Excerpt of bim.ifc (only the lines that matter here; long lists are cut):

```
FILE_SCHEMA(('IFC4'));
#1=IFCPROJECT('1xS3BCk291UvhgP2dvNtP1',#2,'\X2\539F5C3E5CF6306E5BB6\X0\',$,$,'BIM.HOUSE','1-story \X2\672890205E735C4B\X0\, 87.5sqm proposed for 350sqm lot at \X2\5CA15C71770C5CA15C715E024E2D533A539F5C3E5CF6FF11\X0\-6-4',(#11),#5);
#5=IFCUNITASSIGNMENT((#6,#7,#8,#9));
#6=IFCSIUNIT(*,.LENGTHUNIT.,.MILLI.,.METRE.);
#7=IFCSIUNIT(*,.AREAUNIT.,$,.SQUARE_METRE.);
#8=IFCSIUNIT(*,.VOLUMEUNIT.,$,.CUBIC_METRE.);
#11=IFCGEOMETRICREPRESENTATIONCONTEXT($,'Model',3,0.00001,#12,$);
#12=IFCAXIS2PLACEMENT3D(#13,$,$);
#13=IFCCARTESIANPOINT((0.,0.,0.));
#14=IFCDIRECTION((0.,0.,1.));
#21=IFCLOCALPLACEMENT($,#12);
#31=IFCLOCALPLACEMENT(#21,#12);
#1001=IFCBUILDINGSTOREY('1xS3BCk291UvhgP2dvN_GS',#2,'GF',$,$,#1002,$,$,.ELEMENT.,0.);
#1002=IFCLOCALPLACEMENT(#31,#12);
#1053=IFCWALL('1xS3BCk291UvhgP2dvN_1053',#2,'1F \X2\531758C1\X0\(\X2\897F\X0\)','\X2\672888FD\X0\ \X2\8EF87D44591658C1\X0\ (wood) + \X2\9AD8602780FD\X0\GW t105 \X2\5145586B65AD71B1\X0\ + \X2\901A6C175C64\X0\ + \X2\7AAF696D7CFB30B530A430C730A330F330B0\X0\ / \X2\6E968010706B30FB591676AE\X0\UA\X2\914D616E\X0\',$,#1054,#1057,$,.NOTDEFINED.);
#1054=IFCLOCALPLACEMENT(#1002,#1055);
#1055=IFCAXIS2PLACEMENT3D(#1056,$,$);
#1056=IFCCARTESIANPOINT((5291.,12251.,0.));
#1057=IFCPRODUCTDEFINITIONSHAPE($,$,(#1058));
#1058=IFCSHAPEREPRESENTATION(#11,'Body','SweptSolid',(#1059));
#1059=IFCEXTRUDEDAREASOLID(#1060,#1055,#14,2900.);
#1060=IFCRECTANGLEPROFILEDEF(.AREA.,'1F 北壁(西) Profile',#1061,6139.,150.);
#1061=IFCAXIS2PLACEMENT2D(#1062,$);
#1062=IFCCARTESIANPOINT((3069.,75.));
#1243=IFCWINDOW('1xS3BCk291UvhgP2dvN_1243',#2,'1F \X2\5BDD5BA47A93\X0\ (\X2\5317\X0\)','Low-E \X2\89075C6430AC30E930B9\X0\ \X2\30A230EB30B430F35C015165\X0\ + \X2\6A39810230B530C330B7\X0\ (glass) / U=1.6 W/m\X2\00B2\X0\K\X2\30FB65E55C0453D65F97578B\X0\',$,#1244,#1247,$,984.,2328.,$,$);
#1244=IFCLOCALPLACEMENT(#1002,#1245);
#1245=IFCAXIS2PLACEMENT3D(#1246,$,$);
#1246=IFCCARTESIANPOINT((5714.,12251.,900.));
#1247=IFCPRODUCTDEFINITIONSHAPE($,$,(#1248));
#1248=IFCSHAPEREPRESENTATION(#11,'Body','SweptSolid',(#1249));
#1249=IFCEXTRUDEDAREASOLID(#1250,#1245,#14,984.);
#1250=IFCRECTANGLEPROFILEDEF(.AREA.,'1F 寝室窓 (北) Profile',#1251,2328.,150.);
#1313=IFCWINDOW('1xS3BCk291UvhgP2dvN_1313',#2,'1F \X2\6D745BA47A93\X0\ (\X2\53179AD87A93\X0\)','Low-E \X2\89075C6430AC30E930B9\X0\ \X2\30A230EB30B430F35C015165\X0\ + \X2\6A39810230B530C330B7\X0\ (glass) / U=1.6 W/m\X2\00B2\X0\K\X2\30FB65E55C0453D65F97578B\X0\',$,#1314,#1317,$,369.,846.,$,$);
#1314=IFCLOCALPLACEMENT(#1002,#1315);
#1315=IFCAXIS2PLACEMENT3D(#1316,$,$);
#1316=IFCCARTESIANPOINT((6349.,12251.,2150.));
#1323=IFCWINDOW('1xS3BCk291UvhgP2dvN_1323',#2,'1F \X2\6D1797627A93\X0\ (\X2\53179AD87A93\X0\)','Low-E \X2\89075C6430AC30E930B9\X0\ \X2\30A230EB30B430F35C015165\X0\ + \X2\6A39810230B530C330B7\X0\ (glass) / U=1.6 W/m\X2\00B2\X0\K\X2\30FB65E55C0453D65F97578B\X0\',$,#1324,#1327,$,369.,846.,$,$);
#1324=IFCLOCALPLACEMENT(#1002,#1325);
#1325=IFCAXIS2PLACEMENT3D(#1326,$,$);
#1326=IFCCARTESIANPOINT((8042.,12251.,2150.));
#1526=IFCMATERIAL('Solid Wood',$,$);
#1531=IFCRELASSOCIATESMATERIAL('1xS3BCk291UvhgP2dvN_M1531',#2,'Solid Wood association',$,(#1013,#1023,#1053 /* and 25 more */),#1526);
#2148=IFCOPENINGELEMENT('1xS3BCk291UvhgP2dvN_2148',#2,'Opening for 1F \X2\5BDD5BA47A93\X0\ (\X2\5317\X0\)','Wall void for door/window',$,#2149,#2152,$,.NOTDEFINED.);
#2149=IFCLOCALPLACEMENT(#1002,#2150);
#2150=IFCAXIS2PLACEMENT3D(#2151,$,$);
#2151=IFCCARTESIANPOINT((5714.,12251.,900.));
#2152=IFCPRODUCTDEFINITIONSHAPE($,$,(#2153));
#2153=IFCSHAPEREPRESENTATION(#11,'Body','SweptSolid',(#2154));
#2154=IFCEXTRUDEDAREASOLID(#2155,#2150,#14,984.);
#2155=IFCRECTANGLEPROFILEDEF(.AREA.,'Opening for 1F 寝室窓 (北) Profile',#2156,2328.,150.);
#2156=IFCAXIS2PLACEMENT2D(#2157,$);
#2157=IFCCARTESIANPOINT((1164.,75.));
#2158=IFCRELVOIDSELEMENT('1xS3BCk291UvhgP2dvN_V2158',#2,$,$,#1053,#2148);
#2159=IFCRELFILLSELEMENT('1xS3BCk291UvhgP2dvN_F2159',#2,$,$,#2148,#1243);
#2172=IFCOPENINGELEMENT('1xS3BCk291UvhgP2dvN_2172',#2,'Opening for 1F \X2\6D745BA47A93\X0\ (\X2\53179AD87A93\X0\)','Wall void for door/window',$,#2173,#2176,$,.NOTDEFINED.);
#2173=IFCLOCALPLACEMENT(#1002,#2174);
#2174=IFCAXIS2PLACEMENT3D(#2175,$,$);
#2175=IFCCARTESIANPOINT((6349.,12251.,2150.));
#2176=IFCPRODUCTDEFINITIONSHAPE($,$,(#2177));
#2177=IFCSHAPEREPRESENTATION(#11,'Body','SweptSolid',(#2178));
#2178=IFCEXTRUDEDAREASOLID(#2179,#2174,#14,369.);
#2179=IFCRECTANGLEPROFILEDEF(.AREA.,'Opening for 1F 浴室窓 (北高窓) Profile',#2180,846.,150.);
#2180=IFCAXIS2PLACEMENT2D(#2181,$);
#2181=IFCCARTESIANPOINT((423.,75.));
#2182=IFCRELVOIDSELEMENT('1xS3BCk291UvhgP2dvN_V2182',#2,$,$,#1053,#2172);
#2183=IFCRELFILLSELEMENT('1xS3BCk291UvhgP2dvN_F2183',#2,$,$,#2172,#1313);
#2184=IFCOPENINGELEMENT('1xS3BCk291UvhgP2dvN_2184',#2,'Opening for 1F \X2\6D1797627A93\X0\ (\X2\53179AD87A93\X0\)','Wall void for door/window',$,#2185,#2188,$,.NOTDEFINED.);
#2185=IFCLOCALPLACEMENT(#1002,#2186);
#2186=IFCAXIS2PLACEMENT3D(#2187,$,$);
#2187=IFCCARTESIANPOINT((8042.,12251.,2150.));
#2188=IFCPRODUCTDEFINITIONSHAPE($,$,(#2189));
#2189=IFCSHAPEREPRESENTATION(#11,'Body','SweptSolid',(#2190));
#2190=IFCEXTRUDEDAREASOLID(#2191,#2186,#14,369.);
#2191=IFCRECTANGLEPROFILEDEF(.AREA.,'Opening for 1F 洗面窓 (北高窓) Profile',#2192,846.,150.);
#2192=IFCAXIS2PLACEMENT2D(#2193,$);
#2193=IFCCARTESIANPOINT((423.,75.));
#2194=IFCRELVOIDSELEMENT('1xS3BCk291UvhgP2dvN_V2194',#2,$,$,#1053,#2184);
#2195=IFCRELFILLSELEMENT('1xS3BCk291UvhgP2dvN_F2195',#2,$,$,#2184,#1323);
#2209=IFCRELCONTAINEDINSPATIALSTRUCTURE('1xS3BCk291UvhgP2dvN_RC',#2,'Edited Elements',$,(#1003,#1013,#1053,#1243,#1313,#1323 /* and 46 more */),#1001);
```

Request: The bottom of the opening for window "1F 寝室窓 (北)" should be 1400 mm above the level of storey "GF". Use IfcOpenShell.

```python
import numpy as np
import ifcopenshell
import ifcopenshell.api.geometry
import ifcopenshell.geom
import ifcopenshell.util.element
import ifcopenshell.util.placement
import ifcopenshell.util.shape
import ifcopenshell.util.unit

model = ifcopenshell.open("bim.ifc")
unit_scale = ifcopenshell.util.unit.calculate_unit_scale(model)

window = model.by_guid("1xS3BCk291UvhgP2dvN_1243")
opening = window.FillsVoids[0].RelatingOpeningElement
storey = ifcopenshell.util.element.get_container(window, ifc_class="IfcBuildingStorey")
level = ifcopenshell.util.placement.get_local_placement(storey.ObjectPlacement)[2, 3]

# The opening's origin need not be at the sill, so measure its lowest point.
shape = ifcopenshell.geom.create_shape(ifcopenshell.geom.settings(), opening)
bottom = ifcopenshell.util.shape.get_shape_bottom_elevation(shape, shape.geometry) / unit_scale
dz = level + 1.4 / unit_scale - bottom

shift = np.array([0.0, 0.0, dz])
# The window is not placed relative to its opening, so move both.
for product in (opening, window):
    matrix = ifcopenshell.util.placement.get_local_placement(product.ObjectPlacement)
    matrix[:3, 3] += shift
    ifcopenshell.api.geometry.edit_object_placement(model, product=product, matrix=matrix, is_si=False)

print(f"moved by {dz * unit_scale:+.3f} m")

model.write("bim_edited.ifc")
```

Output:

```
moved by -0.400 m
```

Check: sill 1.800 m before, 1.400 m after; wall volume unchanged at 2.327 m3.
